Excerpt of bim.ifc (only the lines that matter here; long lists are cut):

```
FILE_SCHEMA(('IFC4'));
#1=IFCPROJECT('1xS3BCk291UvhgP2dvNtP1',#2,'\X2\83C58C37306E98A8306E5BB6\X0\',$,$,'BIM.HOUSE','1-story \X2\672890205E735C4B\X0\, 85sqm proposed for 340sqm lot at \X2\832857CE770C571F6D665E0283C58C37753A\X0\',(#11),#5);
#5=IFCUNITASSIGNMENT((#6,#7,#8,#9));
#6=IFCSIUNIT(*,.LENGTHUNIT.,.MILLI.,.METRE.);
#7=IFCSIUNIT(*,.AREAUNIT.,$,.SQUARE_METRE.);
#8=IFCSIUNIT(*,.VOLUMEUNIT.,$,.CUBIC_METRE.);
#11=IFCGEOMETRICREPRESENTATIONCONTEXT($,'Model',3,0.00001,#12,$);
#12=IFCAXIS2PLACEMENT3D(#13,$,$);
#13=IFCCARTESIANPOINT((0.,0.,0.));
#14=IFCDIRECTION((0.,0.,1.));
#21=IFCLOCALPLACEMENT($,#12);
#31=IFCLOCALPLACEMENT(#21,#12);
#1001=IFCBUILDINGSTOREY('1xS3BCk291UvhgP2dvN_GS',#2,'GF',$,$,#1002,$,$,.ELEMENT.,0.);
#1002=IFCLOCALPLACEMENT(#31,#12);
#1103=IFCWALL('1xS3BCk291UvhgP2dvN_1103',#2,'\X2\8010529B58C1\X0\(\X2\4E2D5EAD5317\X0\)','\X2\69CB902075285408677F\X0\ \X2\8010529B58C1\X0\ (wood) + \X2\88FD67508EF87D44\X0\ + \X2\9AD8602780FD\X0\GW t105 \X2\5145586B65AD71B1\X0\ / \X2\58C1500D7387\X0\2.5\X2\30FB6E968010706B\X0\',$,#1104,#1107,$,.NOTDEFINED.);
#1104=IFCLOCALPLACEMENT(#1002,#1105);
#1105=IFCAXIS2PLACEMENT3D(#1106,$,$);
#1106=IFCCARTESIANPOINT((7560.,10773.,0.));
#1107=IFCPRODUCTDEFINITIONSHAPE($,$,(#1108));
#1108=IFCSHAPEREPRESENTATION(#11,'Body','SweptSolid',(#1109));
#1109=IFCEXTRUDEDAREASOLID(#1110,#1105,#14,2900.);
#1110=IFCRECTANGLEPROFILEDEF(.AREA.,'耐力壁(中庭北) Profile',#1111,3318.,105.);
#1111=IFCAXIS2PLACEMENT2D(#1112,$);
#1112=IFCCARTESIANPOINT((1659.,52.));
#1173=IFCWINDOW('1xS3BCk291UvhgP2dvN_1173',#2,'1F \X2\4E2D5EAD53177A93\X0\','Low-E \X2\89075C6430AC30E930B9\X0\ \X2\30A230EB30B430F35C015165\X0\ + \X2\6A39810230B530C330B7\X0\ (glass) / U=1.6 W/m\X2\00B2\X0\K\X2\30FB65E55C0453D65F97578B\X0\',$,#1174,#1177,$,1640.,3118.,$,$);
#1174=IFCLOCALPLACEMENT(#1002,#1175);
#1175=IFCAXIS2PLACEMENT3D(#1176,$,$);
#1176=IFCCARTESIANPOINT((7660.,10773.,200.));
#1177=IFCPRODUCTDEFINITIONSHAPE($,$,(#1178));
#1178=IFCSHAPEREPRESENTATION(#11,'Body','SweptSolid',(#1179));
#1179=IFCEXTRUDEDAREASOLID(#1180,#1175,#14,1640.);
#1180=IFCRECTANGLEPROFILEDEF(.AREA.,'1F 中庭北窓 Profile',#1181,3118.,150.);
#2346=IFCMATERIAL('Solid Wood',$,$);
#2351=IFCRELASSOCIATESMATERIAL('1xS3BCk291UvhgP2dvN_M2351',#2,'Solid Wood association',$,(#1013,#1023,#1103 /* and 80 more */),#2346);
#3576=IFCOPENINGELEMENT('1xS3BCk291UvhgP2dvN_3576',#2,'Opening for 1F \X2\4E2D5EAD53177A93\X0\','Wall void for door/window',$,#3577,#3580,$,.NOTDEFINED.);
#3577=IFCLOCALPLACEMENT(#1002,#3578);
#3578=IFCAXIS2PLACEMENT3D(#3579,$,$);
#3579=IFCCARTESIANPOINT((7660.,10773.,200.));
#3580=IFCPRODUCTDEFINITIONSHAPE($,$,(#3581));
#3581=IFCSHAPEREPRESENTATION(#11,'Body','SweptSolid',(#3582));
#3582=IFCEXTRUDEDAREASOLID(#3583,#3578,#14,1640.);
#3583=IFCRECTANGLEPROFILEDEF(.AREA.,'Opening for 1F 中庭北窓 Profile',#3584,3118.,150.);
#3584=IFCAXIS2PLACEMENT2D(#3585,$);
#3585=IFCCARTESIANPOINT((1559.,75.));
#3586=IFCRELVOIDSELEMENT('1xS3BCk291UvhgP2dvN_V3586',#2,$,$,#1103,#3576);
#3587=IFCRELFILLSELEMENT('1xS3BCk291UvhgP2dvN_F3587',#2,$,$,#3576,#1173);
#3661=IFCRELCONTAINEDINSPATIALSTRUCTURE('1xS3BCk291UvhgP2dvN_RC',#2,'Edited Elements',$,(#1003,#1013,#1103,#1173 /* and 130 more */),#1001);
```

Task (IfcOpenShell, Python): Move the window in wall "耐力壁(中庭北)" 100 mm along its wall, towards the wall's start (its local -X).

```python
import ifcopenshell
import ifcopenshell.api.geometry
import ifcopenshell.util.placement
import ifcopenshell.util.unit

model = ifcopenshell.open("bim.ifc")
unit_scale = ifcopenshell.util.unit.calculate_unit_scale(model)

window = model.by_guid("1xS3BCk291UvhgP2dvN_1173")
opening = window.FillsVoids[0].RelatingOpeningElement
wall = opening.VoidsElements[0].RelatingBuildingElement

wall_matrix = ifcopenshell.util.placement.get_local_placement(wall.ObjectPlacement)
shift = wall_matrix[:3, 0] * -0.1 / unit_scale
before = ifcopenshell.util.placement.get_local_placement(window.ObjectPlacement)[:3, 3].copy()

# The window is not placed relative to its opening, so move both.
for product in (opening, window):
    matrix = ifcopenshell.util.placement.get_local_placement(product.ObjectPlacement)
    matrix[:3, 3] += shift
    ifcopenshell.api.geometry.edit_object_placement(model, product=product, matrix=matrix, is_si=False)

after = ifcopenshell.util.placement.get_local_placement(window.ObjectPlacement)[:3, 3]
print("window moved by", (after - before).round(3) + 0.0)

model.write("bim_edited.ifc")
```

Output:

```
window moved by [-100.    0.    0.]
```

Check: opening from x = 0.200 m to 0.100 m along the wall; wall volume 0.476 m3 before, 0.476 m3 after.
